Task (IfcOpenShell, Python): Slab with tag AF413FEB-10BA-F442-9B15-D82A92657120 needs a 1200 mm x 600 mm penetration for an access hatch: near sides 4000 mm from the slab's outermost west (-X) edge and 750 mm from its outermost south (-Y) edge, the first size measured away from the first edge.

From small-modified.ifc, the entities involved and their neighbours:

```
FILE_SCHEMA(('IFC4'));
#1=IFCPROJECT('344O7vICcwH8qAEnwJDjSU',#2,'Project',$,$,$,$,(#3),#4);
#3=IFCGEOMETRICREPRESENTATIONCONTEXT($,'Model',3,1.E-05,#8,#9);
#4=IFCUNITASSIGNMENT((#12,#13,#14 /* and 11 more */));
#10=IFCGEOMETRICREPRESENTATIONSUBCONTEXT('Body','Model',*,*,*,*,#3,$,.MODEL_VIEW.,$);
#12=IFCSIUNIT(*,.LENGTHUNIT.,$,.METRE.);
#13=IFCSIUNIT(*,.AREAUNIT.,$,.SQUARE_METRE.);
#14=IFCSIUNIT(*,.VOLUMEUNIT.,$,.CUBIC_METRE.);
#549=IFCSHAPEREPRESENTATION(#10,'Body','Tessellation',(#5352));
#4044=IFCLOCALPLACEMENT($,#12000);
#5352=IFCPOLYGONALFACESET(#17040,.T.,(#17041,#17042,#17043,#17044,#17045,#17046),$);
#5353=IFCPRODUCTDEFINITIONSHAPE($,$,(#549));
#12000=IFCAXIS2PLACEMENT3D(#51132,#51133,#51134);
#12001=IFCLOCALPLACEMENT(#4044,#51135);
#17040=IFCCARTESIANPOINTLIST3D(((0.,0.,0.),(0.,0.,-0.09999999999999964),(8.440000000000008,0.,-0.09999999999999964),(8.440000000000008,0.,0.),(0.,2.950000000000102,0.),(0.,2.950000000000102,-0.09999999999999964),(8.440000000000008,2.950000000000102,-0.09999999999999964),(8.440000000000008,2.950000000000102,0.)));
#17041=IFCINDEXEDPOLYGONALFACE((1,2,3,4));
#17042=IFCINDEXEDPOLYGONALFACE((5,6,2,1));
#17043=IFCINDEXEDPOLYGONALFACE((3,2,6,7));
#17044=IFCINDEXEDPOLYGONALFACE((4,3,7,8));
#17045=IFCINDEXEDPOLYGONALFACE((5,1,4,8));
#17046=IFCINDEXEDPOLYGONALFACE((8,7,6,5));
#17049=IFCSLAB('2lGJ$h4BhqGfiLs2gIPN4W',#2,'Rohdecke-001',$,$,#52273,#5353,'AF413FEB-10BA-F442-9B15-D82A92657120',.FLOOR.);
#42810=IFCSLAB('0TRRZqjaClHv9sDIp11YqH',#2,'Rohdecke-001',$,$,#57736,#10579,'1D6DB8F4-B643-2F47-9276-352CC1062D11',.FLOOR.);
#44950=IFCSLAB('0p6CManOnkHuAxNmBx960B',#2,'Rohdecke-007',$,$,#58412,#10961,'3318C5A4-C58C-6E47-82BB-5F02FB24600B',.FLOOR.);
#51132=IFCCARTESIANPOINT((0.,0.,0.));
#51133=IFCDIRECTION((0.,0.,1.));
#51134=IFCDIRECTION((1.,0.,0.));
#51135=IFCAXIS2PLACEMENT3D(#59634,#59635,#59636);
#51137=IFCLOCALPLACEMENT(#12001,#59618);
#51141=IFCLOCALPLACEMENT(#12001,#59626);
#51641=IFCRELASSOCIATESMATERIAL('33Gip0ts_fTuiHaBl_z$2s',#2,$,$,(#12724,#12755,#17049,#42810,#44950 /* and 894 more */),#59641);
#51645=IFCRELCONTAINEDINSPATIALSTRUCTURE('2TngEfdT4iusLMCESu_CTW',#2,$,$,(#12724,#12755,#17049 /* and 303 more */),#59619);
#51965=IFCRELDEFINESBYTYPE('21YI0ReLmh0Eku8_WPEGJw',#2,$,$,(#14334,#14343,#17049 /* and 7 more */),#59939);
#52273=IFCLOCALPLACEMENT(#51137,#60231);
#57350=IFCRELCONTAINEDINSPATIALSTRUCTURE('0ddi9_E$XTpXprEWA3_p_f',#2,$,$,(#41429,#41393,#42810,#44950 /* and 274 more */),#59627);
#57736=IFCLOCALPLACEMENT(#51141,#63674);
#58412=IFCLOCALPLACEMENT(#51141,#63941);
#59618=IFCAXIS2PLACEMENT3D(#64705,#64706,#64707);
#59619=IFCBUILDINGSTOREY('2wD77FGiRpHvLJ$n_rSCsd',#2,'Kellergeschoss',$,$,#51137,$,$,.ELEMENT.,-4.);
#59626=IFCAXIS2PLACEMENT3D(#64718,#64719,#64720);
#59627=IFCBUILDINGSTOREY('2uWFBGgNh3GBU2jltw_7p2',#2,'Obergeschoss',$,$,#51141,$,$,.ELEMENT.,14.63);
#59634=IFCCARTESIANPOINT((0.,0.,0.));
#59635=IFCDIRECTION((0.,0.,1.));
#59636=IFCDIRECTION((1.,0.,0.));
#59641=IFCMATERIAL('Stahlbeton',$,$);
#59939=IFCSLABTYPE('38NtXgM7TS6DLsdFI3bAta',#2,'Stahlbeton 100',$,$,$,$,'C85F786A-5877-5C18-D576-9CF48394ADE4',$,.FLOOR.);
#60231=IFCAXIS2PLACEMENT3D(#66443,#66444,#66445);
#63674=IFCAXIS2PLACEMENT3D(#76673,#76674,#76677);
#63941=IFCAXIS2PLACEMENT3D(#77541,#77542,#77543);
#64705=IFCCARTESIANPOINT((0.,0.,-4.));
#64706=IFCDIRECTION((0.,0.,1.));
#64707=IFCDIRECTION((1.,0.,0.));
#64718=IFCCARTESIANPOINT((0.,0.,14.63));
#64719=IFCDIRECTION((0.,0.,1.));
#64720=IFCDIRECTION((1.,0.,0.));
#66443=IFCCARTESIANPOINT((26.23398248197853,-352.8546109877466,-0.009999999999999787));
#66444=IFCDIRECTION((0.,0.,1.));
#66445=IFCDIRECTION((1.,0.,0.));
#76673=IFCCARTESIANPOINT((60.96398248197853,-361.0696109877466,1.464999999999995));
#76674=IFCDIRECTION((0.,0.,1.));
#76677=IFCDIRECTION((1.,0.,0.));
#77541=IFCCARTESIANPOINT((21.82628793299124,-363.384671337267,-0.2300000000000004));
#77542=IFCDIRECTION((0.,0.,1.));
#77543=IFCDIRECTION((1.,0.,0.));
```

```python
import numpy as np
import ifcopenshell
import ifcopenshell.api.feature
import ifcopenshell.api.geometry
import ifcopenshell.api.root
import ifcopenshell.geom
import ifcopenshell.util.placement
import ifcopenshell.util.representation
import ifcopenshell.util.shape
import ifcopenshell.util.unit

model = ifcopenshell.open("small-modified.ifc")
unit_scale = ifcopenshell.util.unit.calculate_unit_scale(model)
settings = ifcopenshell.geom.settings()


def volume(element):
    """Net volume in cubic metres, openings subtracted."""
    shape = ifcopenshell.geom.create_shape(settings, element)
    return ifcopenshell.util.shape.get_volume(shape.geometry)


slab = model.by_guid("2lGJ$h4BhqGfiLs2gIPN4W")
before = volume(slab)

# Extent in the slab's own axes, in metres. The edges named are its -X and -Y sides.
slab_shape = ifcopenshell.geom.create_shape(settings, slab)
vertices = ifcopenshell.util.shape.get_vertices(slab_shape.geometry)
x_min, y_min, bottom = vertices.min(axis=0)
top = vertices[:, 2].max()

opening = ifcopenshell.api.root.create_entity(model, ifc_class="IfcOpeningElement", name="Access hatch opening", predefined_type="OPENING")
context = ifcopenshell.util.representation.get_context(model, "Model", "Body", "MODEL_VIEW")
width, depth = 1.2, 0.6
outline = [(0.0, 0.0), (width, 0.0), (width, depth), (0.0, depth), (0.0, 0.0)]
# Overshoot both faces by 50 mm so the cut is clean.
shape = ifcopenshell.api.geometry.add_slab_representation(
    model, context=context, depth=top - bottom + 0.1, polyline=outline
)
ifcopenshell.api.geometry.assign_representation(model, product=opening, representation=shape)

matrix = ifcopenshell.util.placement.get_local_placement(slab.ObjectPlacement)
matrix[:, 3] = matrix @ np.append(np.array([x_min + 4, y_min + 0.75, bottom - 0.05]) / unit_scale, 1.0)
ifcopenshell.api.geometry.edit_object_placement(model, product=opening, matrix=matrix, is_si=False)
ifcopenshell.api.feature.add_feature(model, feature=opening, element=slab)

after = volume(slab)

print(f"slab volume {before:.3f} -> {after:.3f} m3")

model.write("small-modified_v2.ifc")
```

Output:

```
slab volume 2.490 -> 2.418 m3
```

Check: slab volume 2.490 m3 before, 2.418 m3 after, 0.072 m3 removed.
